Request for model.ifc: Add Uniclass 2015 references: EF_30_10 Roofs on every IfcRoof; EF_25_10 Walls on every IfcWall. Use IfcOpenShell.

First a look at what the model holds.

```python
import ifcopenshell

model = ifcopenshell.open("model.ifc")
print(model.schema)
print("classifications:", [c.Name for c in model.by_type("IfcClassification")])
for ifc_class in ("IfcDoor", "IfcRoof", "IfcStair", "IfcWall", "IfcWindow"):
    print(ifc_class, len(model.by_type(ifc_class)))
```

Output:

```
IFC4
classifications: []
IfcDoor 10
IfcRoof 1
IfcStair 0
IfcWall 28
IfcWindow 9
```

```python
import ifcopenshell
import ifcopenshell.api.classification

model = ifcopenshell.open("model.ifc")

system = ifcopenshell.api.classification.add_classification(model, classification="Uniclass 2015")

codes = {
    "IfcRoof": ("EF_30_10", "Roofs"),
    "IfcWall": ("EF_25_10", "Walls"),
}
for ifc_class, (code, name) in codes.items():
    products = model.by_type(ifc_class)
    ifcopenshell.api.classification.add_reference(
        model, products=products, classification=system, identification=code, name=name
    )
    print(code, len(products))

model.write("model-out.ifc")
```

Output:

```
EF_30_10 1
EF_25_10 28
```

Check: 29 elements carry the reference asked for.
